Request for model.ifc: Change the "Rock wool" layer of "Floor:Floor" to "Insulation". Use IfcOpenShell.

First a look at what the model holds.

```python
import ifcopenshell
import ifcopenshell.util.element

model = ifcopenshell.open("model.ifc")
print(model.schema)
for layer_set in model.by_type("IfcMaterialLayerSet"):
    if layer_set.LayerSetName == "Floor:Floor":
        for layer in layer_set.MaterialLayers:
            print(layer.id(), layer.Material and layer.Material.Name, layer.LayerThickness, sep=" | ")
        print(len(ifcopenshell.util.element.get_elements_by_material(model, layer_set)), "elements and types use it")
print(sorted(m.Name for m in model.by_type("IfcMaterial") if m.Name)[:60])
```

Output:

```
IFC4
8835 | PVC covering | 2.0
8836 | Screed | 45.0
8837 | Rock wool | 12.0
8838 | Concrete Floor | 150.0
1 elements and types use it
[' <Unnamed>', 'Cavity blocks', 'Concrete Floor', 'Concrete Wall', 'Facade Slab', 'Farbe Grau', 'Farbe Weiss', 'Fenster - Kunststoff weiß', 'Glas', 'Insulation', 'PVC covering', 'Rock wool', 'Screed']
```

```python
import ifcopenshell
import ifcopenshell.api.material

model = ifcopenshell.open("model.ifc")

layer_set = next(s for s in model.by_type("IfcMaterialLayerSet") if s.LayerSetName == "Floor:Floor")
layer = next(l for l in layer_set.MaterialLayers if l.Material and l.Material.Name == "Rock wool")
material = next(m for m in model.by_type("IfcMaterial") if m.Name == "Insulation")

# Point this one layer at the other material; renaming the old one would change it everywhere.
ifcopenshell.api.material.edit_layer(model, layer=layer, attributes={}, material=material)

print([l.Material.Name if l.Material else None for l in layer_set.MaterialLayers])

model.write("model_v2.ifc")
```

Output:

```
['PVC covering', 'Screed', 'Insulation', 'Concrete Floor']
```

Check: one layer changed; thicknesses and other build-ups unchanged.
